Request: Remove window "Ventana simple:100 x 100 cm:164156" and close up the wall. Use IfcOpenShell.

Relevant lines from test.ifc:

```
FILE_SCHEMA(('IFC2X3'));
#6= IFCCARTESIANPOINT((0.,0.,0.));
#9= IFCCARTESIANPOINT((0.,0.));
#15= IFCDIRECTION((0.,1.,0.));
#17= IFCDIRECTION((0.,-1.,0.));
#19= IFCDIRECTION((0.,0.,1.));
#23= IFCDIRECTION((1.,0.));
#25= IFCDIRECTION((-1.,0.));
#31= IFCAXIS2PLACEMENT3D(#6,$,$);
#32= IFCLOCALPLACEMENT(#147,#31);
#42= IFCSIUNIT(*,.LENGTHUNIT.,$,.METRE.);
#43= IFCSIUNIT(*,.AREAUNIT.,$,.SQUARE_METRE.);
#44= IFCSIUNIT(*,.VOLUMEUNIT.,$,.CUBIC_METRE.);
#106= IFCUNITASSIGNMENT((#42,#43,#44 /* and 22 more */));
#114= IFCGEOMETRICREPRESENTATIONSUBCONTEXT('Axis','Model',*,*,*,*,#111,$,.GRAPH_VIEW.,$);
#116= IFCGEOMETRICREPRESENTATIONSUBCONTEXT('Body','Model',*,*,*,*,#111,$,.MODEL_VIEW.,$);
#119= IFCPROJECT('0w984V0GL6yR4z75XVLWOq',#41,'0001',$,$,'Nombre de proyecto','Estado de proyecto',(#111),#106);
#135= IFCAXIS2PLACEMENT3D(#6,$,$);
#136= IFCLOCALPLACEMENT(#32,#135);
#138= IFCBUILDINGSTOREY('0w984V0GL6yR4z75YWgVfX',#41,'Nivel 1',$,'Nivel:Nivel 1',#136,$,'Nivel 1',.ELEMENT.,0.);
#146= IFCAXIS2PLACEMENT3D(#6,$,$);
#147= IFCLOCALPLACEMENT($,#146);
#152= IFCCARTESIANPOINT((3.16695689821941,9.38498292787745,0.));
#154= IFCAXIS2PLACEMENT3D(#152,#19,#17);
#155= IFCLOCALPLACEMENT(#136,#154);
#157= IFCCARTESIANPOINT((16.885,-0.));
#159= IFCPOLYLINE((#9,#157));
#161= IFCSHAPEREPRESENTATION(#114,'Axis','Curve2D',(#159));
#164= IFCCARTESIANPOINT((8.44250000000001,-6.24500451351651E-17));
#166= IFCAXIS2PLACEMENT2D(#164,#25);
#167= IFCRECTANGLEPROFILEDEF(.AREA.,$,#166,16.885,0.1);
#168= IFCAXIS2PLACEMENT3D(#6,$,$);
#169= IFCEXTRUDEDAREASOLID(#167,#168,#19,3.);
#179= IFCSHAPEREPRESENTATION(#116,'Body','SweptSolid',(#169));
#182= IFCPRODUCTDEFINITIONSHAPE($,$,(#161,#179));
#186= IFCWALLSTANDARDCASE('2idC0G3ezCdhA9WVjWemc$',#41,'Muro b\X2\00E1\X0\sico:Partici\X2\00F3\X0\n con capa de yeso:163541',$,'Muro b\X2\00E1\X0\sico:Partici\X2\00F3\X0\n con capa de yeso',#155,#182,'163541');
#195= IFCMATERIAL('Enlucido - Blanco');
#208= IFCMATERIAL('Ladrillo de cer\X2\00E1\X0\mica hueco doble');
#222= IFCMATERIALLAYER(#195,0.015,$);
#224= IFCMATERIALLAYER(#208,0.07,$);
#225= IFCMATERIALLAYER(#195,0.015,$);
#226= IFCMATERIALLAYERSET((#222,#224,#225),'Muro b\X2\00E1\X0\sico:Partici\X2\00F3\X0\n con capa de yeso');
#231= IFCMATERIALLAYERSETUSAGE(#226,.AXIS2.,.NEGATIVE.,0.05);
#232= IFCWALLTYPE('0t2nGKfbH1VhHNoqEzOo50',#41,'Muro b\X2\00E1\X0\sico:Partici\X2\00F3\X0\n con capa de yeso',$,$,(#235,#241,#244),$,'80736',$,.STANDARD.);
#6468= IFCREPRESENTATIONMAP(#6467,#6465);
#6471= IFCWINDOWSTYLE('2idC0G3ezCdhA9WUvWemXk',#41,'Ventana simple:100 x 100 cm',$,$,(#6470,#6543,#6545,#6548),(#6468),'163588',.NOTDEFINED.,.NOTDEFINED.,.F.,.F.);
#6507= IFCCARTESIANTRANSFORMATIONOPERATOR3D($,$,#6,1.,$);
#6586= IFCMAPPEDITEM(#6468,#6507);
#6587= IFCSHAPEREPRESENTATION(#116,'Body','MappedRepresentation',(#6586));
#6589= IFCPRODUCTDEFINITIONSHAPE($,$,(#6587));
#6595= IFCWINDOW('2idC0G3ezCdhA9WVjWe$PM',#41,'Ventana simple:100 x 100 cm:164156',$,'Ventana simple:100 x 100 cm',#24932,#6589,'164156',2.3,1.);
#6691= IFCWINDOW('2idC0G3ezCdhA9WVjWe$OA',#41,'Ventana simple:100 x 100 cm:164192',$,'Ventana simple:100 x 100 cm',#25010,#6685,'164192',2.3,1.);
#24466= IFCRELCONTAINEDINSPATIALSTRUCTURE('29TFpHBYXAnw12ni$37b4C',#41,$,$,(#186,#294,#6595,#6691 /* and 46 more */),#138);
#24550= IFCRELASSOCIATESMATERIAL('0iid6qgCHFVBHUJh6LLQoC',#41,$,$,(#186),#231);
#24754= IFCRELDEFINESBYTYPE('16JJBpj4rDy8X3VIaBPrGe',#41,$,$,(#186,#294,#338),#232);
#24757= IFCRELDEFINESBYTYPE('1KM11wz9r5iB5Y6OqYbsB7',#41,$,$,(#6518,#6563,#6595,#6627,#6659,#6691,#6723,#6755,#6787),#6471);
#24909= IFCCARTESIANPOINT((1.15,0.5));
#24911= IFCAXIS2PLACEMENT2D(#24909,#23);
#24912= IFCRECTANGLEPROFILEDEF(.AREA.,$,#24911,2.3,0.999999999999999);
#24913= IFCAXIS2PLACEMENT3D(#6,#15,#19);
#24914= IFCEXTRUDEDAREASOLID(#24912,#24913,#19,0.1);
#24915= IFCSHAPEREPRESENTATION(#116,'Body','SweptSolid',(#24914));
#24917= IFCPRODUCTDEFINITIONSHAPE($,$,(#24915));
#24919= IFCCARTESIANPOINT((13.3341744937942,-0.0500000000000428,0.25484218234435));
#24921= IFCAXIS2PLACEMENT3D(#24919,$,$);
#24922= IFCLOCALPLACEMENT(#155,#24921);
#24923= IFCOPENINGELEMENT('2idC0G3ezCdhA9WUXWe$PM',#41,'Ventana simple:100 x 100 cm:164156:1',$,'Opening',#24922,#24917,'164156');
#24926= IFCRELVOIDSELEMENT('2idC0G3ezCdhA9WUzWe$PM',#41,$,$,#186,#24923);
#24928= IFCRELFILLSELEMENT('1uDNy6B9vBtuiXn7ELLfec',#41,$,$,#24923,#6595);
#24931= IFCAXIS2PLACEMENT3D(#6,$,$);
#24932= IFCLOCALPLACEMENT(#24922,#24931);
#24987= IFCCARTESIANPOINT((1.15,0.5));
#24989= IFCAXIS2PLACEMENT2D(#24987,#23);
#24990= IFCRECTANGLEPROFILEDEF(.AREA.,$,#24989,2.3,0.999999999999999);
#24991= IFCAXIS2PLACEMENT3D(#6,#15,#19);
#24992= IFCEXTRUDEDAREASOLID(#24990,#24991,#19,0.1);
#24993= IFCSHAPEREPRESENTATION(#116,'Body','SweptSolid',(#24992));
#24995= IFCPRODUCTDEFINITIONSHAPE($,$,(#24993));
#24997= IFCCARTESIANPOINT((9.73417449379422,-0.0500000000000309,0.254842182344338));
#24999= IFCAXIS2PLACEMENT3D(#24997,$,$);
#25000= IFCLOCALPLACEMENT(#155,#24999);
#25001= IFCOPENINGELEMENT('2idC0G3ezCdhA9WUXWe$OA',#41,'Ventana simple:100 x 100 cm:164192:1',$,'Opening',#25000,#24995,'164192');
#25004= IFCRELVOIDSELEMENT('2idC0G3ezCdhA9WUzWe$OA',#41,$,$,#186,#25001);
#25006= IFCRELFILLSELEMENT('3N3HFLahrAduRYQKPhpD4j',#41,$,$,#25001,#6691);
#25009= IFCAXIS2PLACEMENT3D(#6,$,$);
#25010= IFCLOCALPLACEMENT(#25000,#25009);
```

```python
import ifcopenshell
import ifcopenshell.api.feature
import ifcopenshell.api.root
import ifcopenshell.geom
import ifcopenshell.util.shape

model = ifcopenshell.open("test.ifc")
settings = ifcopenshell.geom.settings()


def volume(element):
    """Net volume in cubic metres, openings subtracted."""
    shape = ifcopenshell.geom.create_shape(settings, element)
    return ifcopenshell.util.shape.get_volume(shape.geometry)


window = model.by_guid("2idC0G3ezCdhA9WVjWe$PM")
opening = window.FillsVoids[0].RelatingOpeningElement
wall = opening.VoidsElements[0].RelatingBuildingElement
before = volume(wall)

ifcopenshell.api.root.remove_product(model, product=window)
ifcopenshell.api.feature.remove_feature(model, feature=opening)

after = volume(wall)

print(f"wall volume {before:.3f} -> {after:.3f} m3")

model.write("test-out.ifc")
```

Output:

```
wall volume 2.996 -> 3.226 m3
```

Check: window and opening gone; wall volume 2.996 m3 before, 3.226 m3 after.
